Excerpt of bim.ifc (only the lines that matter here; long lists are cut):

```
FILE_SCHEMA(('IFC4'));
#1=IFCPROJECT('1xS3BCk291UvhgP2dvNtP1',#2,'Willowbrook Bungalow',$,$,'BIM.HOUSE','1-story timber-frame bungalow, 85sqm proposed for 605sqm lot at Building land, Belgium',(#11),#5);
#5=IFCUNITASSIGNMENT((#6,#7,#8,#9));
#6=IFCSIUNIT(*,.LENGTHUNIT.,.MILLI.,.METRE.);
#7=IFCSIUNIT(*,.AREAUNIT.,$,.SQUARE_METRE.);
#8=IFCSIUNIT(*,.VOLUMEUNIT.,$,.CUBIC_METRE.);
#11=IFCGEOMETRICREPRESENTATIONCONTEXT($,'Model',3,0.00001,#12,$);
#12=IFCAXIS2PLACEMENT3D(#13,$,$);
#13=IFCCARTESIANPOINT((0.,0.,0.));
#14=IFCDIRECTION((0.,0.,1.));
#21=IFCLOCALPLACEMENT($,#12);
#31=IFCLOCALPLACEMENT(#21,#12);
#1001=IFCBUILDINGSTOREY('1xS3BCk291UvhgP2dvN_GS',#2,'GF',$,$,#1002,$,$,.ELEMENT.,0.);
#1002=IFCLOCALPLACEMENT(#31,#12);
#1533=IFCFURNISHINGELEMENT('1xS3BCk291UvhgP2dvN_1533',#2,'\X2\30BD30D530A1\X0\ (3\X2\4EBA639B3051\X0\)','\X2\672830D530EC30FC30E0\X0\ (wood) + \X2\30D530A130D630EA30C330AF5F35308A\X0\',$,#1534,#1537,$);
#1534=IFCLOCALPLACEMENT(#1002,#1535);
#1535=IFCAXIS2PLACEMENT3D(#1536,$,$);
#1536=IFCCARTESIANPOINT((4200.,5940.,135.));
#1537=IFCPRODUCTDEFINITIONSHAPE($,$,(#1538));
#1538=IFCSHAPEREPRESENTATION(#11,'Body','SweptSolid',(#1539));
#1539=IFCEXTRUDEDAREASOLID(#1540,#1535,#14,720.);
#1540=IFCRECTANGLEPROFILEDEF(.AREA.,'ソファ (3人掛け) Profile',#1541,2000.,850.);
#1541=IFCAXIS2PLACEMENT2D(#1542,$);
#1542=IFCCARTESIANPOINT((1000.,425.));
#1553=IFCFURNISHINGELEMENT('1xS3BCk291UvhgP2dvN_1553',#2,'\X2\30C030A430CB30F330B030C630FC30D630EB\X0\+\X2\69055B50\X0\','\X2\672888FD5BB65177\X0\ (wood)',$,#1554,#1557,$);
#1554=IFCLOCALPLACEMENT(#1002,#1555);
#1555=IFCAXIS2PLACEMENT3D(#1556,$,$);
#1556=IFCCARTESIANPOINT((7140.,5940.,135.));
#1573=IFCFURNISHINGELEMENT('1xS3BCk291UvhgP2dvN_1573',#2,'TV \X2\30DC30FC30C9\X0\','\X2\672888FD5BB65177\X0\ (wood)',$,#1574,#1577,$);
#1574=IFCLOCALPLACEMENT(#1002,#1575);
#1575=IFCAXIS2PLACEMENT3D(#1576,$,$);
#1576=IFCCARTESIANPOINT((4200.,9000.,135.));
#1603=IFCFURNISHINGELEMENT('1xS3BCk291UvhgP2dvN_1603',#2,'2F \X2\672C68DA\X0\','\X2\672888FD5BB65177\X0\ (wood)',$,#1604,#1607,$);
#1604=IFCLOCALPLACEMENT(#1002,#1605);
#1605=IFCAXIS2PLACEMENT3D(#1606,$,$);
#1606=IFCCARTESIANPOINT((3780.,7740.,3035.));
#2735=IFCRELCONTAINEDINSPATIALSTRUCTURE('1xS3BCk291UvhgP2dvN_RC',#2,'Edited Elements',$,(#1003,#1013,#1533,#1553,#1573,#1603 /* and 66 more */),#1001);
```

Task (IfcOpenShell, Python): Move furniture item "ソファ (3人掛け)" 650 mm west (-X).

```python
import ifcopenshell
import ifcopenshell.api.geometry
import ifcopenshell.util.placement

model = ifcopenshell.open("bim.ifc")

item = model.by_id(1533)
matrix = ifcopenshell.util.placement.get_local_placement(item.ObjectPlacement)
matrix[0, 3] -= 650.0
ifcopenshell.api.geometry.edit_object_placement(model, product=item, matrix=matrix, is_si=False)

print(ifcopenshell.util.placement.get_local_placement(item.ObjectPlacement).round(3) + 0.0)

model.write("bim_rev.ifc")
```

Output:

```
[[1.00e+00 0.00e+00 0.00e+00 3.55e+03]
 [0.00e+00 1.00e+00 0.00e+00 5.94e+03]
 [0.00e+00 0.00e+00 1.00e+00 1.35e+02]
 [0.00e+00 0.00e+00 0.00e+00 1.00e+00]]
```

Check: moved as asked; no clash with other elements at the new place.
